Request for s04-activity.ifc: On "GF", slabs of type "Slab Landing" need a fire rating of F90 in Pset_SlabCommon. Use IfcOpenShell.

First a look at what the model holds.

```python
import ifcopenshell
import ifcopenshell.util.element

model = ifcopenshell.open("s04-activity.ifc")
print(model.schema)
storey = next(s for s in model.by_type("IfcBuildingStorey") if s.Name == "GF")
slabs = [e for e in ifcopenshell.util.element.get_decomposition(storey) if e.is_a("IfcSlab")]
seen = {}
for e in slabs:
    element_type = ifcopenshell.util.element.get_type(e)
    key = (element_type.Name if element_type != e and element_type else None, ifcopenshell.util.element.get_pset(e, "Pset_SlabCommon", "FireRating"))
    seen[key] = seen.get(key, 0) + 1
for (name, value), count in sorted(seen.items(), key=str):
    print(count, "x", name, "|", value)
```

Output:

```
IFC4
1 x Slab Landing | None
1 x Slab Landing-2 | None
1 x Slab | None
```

```python
import ifcopenshell
import ifcopenshell.api.pset
import ifcopenshell.util.element

model = ifcopenshell.open("s04-activity.ifc")

storey = next(s for s in model.by_type("IfcBuildingStorey") if s.Name == "GF")
slabs = [e for e in ifcopenshell.util.element.get_decomposition(storey) if e.is_a("IfcSlab")]

count = 0
for e in slabs:
    element_type = ifcopenshell.util.element.get_type(e)
    if element_type in (None, e) or element_type.Name != "Slab Landing":
        continue
    # add_pset returns the element's existing set when there is one.
    pset = ifcopenshell.api.pset.add_pset(model, product=e, name="Pset_SlabCommon")
    ifcopenshell.api.pset.edit_pset(model, pset=pset, properties={"FireRating": "F90"})
    count += 1

print(count, "slabs updated")

model.write("s04-activity_updated.ifc")
```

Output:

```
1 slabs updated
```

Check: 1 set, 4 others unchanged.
